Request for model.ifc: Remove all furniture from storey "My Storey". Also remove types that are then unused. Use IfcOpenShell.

First a look at what the model holds.

```python
import ifcopenshell
import ifcopenshell.util.element

model = ifcopenshell.open("model.ifc")
print(model.schema)
storey = next(s for s in model.by_type("IfcBuildingStorey") if s.Name == "My Storey")
furniture = [e for e in ifcopenshell.util.element.get_decomposition(storey) if e.is_a("IfcFurnishingElement")]
seen = {}
for e in furniture:
    element_type = ifcopenshell.util.element.get_type(e)
    name = element_type.Name if element_type not in (None, e) else None
    seen[name] = seen.get(name, 0) + 1
for name, count in sorted(seen.items(), key=str):
    print(count, "x", name)
```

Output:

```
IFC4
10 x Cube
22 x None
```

```python
import ifcopenshell
import ifcopenshell.api.root
import ifcopenshell.util.element

model = ifcopenshell.open("model.ifc")

storey = next(s for s in model.by_type("IfcBuildingStorey") if s.Name == "My Storey")
furniture = [e for e in ifcopenshell.util.element.get_decomposition(storey) if e.is_a("IfcFurnishingElement")]
types = {ifcopenshell.util.element.get_type(e) for e in furniture} - {None, *furniture}

for e in furniture:
    ifcopenshell.api.root.remove_product(model, product=e)
print(len(furniture), "removed")

unused = [t for t in types if not ifcopenshell.util.element.get_types(t)]
for t in unused:
    ifcopenshell.api.root.remove_product(model, product=t)
print(len(unused), "unused types removed")

model.write("model_rev.ifc")
```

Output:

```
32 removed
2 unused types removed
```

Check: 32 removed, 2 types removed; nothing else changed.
